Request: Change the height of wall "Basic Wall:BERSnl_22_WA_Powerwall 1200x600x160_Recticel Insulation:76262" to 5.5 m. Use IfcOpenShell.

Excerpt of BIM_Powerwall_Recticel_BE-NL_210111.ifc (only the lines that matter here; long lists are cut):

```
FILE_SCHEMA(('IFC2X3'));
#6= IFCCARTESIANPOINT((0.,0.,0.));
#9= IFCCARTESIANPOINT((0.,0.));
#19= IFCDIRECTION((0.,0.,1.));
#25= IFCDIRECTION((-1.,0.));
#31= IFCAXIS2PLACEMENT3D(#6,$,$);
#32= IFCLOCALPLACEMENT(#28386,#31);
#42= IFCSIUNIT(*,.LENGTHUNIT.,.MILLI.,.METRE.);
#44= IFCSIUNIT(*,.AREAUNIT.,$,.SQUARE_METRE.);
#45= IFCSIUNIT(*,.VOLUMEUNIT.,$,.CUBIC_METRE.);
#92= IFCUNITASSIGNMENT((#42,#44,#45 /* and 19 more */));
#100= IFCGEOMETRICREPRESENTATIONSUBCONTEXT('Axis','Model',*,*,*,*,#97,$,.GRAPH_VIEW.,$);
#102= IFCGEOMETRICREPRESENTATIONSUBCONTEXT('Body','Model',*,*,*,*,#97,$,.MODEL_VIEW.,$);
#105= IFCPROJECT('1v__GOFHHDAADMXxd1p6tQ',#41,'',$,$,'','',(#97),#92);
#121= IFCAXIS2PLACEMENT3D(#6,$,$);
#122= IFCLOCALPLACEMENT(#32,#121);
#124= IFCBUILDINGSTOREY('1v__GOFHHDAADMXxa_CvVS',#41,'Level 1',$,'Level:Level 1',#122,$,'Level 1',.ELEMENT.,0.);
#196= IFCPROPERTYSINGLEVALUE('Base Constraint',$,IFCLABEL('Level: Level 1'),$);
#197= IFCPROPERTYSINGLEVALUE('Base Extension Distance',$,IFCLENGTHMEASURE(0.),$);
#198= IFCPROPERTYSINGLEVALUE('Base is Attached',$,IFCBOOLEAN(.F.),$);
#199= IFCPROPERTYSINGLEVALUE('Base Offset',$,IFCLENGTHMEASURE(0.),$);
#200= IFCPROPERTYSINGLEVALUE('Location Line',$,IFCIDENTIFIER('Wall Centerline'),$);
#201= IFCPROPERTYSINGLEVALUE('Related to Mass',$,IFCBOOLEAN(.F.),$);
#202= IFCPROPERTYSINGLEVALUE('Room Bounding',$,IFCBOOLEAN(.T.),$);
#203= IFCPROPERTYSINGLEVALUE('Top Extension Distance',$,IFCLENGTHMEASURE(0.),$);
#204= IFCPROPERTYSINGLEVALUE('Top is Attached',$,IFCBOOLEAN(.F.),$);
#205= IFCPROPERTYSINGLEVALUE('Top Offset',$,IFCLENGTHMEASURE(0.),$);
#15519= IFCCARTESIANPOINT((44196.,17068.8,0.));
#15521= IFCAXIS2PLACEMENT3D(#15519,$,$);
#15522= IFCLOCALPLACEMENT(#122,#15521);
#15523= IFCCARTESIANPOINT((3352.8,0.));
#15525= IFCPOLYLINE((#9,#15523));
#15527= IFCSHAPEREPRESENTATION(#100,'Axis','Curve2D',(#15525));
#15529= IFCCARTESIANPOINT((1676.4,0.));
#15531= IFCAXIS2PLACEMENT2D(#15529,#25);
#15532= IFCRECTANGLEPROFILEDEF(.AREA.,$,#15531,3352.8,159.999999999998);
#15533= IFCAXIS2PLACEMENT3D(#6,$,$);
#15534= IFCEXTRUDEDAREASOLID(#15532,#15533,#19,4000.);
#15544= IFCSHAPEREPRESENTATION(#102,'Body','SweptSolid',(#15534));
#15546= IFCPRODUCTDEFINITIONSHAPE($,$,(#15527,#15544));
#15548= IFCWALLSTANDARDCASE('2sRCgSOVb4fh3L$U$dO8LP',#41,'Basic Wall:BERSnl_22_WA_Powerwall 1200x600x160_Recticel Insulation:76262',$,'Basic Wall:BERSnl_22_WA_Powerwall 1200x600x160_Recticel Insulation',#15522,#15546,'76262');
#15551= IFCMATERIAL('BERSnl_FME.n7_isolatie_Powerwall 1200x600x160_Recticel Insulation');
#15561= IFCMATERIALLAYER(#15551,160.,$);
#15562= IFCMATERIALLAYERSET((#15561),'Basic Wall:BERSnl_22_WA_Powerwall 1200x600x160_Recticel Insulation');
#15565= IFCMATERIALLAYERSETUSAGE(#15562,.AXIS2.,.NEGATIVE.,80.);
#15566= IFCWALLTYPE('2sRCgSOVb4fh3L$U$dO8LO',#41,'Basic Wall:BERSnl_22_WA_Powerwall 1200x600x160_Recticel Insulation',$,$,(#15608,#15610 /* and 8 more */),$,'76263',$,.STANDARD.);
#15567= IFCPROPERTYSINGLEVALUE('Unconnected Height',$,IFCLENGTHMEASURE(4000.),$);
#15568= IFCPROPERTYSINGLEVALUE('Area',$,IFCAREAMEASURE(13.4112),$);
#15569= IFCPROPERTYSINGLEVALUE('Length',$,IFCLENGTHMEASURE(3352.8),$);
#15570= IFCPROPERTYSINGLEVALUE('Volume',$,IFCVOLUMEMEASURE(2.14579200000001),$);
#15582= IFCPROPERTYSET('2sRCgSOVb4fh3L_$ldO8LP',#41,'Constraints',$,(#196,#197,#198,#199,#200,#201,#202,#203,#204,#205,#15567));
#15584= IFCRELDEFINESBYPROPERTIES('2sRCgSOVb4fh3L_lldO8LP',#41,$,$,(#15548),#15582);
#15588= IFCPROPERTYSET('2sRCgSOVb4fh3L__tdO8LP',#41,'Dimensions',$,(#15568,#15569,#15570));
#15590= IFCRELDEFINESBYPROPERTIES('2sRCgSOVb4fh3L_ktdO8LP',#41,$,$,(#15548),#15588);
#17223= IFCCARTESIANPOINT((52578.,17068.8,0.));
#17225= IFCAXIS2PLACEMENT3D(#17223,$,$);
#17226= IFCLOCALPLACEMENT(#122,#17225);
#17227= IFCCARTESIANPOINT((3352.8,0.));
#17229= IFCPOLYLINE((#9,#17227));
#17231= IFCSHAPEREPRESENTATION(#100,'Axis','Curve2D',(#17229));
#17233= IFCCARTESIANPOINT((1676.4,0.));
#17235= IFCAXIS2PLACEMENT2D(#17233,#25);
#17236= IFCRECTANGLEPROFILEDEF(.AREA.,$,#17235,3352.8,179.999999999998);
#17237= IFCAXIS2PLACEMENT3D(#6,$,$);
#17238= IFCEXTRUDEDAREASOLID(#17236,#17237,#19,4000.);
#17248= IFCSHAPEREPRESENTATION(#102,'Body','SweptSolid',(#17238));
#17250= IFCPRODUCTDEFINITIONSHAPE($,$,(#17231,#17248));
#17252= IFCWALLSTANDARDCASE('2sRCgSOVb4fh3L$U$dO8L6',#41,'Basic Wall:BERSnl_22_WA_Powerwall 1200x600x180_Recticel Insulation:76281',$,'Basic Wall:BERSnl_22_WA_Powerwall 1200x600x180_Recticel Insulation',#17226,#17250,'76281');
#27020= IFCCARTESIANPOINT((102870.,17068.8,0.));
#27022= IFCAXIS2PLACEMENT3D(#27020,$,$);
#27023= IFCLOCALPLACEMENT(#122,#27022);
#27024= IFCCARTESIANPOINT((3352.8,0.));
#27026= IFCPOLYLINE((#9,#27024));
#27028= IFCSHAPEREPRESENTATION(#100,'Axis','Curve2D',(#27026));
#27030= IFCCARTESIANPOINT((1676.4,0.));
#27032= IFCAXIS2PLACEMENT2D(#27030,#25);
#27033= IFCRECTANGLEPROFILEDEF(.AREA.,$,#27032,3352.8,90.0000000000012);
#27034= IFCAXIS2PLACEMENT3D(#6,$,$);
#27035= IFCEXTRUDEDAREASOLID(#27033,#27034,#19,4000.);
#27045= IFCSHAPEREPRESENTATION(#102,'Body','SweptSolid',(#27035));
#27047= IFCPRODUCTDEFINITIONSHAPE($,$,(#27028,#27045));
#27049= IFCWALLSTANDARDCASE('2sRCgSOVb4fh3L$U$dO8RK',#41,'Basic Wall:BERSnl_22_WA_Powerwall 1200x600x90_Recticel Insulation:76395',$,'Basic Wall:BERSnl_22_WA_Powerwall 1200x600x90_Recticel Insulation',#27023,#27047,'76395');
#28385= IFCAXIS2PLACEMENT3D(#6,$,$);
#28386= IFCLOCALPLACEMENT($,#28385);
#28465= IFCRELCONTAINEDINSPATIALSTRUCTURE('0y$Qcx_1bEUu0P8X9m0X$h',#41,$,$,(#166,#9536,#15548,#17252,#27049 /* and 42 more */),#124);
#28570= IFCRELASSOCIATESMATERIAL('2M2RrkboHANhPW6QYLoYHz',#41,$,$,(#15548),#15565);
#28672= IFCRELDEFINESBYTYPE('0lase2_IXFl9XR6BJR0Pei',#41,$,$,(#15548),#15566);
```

```python
import ifcopenshell
import ifcopenshell.api.pset
import ifcopenshell.geom
import ifcopenshell.util.element
import ifcopenshell.util.representation
import ifcopenshell.util.shape
import ifcopenshell.util.unit

model = ifcopenshell.open("BIM_Powerwall_Recticel_BE-NL_210111.ifc")
area_scale = ifcopenshell.util.unit.calculate_unit_scale(model, "AREAUNIT")
volume_scale = ifcopenshell.util.unit.calculate_unit_scale(model, "VOLUMEUNIT")
settings = ifcopenshell.geom.settings()


def volume(element):
    """Net volume in cubic metres, openings subtracted."""
    shape = ifcopenshell.geom.create_shape(settings, element)
    return ifcopenshell.util.shape.get_volume(shape.geometry)


wall = model.by_id(15548)
before = volume(wall)

body = ifcopenshell.util.representation.get_representation(wall, "Model", "Body")
solid = body.Items[0]
old_height = solid.Depth
solid.Depth = 5500.0
after = volume(wall)
thickness = 0.16  # wall thickness in metres

# Update the stored height, areas and volumes.
pset = model.by_id(ifcopenshell.util.element.get_pset(wall, "Constraints", should_inherit=False)["id"])
ifcopenshell.api.pset.edit_pset(model, pset=pset, properties={
    "Unconnected Height": model.create_entity("IfcLengthMeasure", solid.Depth),
})
pset = model.by_id(ifcopenshell.util.element.get_pset(wall, "Dimensions", should_inherit=False)["id"])
ifcopenshell.api.pset.edit_pset(model, pset=pset, properties={
    "Area": model.create_entity("IfcAreaMeasure", after / thickness / area_scale),
    "Volume": model.create_entity("IfcVolumeMeasure", after / volume_scale),
})

print(f"height {old_height:g} -> {solid.Depth:g}, volume {before:.3f} -> {after:.3f} m3")

model.write("BIM_Powerwall_Recticel_BE-NL_210111-out.ifc")
```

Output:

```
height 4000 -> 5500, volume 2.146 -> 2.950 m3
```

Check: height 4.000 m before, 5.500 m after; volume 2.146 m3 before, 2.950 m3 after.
